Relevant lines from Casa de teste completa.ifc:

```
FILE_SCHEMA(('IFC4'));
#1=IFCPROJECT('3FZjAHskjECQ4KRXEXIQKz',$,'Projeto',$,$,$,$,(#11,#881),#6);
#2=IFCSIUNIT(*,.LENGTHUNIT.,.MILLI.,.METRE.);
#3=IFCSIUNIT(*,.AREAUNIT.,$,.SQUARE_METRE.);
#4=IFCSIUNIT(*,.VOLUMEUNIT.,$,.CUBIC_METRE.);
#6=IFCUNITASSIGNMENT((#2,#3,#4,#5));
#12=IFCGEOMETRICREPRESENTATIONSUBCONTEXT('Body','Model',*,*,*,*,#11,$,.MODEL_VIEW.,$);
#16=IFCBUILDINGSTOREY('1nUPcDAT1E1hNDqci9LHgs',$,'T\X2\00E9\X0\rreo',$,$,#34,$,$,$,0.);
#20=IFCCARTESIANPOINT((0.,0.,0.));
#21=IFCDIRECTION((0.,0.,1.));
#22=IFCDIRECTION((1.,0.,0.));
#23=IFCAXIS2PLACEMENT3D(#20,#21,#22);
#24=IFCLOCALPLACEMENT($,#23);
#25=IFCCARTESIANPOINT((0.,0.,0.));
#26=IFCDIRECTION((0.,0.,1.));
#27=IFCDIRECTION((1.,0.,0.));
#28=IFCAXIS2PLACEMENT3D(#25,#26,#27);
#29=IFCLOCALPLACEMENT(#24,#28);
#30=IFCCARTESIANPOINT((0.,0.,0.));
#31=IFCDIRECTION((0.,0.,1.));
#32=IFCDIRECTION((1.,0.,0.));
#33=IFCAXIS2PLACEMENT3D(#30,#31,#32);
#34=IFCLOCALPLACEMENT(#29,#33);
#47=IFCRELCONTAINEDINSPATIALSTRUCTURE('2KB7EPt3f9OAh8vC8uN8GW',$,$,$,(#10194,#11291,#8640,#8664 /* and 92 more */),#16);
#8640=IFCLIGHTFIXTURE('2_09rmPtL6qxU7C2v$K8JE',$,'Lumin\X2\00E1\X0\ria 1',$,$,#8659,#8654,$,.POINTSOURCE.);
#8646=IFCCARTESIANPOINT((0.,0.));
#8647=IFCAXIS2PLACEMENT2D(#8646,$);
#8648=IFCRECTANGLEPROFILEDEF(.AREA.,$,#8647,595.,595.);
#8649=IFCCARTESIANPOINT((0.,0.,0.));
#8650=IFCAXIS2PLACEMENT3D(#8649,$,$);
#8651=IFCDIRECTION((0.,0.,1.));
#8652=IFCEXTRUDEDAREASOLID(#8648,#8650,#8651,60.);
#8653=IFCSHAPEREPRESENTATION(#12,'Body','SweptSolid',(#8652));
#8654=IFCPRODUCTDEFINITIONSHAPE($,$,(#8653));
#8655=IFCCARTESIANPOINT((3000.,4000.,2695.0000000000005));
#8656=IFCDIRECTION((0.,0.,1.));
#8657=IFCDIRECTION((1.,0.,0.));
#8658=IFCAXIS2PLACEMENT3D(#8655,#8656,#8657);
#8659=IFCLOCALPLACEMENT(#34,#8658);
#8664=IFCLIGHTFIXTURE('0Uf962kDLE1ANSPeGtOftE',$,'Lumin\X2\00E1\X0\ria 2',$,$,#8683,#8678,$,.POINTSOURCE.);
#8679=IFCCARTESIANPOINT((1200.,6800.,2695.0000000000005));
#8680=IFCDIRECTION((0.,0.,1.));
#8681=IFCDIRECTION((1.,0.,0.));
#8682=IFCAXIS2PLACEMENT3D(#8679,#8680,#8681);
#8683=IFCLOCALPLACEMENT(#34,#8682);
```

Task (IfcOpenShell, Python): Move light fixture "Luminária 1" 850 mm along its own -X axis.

```python
import ifcopenshell
import ifcopenshell.api.geometry
import ifcopenshell.util.placement
import ifcopenshell.util.unit

model = ifcopenshell.open("Casa de teste completa.ifc")
unit_scale = ifcopenshell.util.unit.calculate_unit_scale(model)

item = model.by_id(8640)
matrix = ifcopenshell.util.placement.get_local_placement(item.ObjectPlacement)
matrix[:3, 3] -= matrix[:3, 0] * 0.85 / unit_scale
ifcopenshell.api.geometry.edit_object_placement(model, product=item, matrix=matrix, is_si=False)

print(ifcopenshell.util.placement.get_local_placement(item.ObjectPlacement).round(3) + 0.0)

model.write("Casa de teste completa_rev.ifc")
```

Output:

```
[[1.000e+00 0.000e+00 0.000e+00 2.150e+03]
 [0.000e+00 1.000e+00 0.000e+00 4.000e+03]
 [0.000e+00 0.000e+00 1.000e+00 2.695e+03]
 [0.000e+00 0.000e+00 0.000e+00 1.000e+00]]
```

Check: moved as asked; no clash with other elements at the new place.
